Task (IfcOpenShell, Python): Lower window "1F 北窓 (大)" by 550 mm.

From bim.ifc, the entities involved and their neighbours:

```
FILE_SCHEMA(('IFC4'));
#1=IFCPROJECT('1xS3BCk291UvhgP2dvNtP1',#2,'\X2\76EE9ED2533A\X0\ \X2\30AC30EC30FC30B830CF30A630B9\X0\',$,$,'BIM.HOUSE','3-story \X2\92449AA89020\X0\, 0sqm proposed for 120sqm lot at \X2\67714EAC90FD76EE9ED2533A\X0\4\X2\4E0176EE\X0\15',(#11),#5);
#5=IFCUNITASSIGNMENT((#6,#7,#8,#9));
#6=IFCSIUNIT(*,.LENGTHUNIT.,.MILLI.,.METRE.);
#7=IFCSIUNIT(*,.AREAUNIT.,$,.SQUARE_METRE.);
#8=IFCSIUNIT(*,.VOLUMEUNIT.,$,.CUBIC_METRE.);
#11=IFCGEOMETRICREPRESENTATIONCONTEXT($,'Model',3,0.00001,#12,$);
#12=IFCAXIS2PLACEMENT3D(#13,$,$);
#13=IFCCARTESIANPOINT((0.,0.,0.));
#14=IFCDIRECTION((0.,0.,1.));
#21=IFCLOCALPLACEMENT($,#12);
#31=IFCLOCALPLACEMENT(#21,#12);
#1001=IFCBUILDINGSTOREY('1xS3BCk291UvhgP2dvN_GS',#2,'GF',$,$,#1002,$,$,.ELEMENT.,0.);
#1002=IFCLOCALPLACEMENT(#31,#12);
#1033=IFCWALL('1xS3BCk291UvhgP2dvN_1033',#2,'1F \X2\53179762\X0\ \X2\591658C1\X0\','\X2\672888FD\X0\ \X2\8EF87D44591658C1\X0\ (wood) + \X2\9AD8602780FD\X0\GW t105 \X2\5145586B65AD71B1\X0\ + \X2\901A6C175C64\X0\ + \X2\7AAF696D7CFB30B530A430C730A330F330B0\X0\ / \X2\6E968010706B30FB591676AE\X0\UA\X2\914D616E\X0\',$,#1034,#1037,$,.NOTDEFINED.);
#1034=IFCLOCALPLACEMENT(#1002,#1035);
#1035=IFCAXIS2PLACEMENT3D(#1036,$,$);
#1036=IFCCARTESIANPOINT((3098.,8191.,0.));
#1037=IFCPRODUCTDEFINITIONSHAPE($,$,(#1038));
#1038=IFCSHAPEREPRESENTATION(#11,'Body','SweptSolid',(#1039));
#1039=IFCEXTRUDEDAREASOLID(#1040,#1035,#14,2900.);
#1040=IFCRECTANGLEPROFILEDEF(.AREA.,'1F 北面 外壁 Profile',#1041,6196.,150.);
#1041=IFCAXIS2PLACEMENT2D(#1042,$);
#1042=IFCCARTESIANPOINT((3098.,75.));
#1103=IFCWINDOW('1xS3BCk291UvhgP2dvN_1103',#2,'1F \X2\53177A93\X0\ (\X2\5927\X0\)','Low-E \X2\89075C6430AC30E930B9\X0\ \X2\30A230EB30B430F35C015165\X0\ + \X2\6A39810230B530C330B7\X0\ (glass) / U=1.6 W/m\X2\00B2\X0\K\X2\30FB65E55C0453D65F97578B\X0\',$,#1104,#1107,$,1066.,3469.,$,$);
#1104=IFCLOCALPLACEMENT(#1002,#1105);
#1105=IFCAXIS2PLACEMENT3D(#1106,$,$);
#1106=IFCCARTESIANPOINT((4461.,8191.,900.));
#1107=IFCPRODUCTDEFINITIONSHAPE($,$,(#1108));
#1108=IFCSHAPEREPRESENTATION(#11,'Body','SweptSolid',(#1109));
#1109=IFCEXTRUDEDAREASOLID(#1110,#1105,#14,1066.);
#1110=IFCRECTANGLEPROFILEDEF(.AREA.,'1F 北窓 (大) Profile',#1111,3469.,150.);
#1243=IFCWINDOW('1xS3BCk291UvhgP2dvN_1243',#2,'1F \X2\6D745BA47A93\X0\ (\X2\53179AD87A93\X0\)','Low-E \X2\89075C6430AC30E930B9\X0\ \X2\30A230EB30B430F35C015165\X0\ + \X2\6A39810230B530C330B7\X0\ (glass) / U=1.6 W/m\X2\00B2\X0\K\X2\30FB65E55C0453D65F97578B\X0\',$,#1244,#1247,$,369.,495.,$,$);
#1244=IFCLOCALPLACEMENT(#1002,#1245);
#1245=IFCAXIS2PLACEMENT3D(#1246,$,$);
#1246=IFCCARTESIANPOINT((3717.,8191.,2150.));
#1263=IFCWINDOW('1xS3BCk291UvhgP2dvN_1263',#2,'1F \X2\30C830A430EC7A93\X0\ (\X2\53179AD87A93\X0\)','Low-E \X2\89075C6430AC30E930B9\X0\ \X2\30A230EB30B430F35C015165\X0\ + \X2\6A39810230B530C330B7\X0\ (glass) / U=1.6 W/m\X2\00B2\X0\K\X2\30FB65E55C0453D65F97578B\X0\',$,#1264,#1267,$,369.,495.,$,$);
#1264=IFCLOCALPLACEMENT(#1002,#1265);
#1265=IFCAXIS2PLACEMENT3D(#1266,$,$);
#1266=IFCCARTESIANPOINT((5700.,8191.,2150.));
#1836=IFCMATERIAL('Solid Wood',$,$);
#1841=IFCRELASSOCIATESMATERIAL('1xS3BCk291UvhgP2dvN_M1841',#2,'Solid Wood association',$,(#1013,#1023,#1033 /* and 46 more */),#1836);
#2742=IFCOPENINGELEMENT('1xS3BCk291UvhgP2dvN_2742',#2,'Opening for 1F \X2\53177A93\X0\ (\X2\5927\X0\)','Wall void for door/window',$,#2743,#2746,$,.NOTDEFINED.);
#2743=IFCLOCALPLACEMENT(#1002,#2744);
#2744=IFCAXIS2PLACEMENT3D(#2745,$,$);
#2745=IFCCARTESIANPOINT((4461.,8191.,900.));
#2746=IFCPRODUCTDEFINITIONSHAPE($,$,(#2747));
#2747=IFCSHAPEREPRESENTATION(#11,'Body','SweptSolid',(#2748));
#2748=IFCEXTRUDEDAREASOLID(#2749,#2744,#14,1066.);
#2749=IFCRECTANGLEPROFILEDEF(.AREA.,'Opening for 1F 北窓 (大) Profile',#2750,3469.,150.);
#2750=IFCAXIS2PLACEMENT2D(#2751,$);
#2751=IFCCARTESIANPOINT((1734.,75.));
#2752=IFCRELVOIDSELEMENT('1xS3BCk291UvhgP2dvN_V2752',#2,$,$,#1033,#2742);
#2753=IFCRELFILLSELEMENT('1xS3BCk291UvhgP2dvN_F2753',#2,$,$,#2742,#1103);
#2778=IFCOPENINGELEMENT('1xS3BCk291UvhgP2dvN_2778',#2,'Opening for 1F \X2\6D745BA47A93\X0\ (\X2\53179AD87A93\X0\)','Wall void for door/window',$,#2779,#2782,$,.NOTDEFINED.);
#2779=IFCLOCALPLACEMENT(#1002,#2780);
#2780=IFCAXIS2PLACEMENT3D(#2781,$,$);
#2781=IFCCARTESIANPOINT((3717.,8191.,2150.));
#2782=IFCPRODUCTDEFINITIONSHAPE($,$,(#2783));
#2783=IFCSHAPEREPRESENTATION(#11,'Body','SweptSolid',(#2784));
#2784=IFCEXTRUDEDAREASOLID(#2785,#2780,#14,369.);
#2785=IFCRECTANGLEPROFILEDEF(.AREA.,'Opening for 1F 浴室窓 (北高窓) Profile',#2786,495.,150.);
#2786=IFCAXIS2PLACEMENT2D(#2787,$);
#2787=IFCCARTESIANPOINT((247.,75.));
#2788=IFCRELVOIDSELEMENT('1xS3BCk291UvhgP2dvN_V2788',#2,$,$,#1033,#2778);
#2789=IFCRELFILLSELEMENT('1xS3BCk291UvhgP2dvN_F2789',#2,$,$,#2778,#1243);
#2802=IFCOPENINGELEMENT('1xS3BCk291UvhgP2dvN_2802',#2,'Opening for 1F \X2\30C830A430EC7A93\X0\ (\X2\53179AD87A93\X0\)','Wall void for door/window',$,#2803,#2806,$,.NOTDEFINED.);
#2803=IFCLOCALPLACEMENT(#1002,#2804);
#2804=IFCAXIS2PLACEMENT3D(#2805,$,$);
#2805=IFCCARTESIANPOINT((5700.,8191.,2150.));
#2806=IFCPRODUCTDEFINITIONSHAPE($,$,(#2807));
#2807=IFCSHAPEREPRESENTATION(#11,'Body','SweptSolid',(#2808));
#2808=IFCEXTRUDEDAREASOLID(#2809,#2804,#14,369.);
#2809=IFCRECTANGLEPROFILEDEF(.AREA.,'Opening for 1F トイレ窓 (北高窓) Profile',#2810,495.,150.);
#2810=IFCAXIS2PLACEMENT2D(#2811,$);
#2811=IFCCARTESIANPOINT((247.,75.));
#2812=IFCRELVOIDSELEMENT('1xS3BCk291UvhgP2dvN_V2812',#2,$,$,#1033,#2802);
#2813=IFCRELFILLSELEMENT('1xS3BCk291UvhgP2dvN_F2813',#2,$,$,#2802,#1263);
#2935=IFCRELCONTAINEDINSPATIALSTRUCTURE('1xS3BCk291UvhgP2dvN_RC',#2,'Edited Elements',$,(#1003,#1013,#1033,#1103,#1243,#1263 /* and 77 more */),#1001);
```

```python
import numpy as np
import ifcopenshell
import ifcopenshell.api.geometry
import ifcopenshell.util.placement
import ifcopenshell.util.unit

model = ifcopenshell.open("bim.ifc")
unit_scale = ifcopenshell.util.unit.calculate_unit_scale(model)

window = model.by_id(1103)
opening = window.FillsVoids[0].RelatingOpeningElement
dz = -0.55 / unit_scale

shift = np.array([0.0, 0.0, dz])
# The window is not placed relative to its opening, so move both.
for product in (opening, window):
    matrix = ifcopenshell.util.placement.get_local_placement(product.ObjectPlacement)
    matrix[:3, 3] += shift
    ifcopenshell.api.geometry.edit_object_placement(model, product=product, matrix=matrix, is_si=False)

print(f"moved by {dz * unit_scale:+.3f} m")

model.write("bim_rev.ifc")
```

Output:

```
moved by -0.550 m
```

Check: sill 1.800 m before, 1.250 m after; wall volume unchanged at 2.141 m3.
